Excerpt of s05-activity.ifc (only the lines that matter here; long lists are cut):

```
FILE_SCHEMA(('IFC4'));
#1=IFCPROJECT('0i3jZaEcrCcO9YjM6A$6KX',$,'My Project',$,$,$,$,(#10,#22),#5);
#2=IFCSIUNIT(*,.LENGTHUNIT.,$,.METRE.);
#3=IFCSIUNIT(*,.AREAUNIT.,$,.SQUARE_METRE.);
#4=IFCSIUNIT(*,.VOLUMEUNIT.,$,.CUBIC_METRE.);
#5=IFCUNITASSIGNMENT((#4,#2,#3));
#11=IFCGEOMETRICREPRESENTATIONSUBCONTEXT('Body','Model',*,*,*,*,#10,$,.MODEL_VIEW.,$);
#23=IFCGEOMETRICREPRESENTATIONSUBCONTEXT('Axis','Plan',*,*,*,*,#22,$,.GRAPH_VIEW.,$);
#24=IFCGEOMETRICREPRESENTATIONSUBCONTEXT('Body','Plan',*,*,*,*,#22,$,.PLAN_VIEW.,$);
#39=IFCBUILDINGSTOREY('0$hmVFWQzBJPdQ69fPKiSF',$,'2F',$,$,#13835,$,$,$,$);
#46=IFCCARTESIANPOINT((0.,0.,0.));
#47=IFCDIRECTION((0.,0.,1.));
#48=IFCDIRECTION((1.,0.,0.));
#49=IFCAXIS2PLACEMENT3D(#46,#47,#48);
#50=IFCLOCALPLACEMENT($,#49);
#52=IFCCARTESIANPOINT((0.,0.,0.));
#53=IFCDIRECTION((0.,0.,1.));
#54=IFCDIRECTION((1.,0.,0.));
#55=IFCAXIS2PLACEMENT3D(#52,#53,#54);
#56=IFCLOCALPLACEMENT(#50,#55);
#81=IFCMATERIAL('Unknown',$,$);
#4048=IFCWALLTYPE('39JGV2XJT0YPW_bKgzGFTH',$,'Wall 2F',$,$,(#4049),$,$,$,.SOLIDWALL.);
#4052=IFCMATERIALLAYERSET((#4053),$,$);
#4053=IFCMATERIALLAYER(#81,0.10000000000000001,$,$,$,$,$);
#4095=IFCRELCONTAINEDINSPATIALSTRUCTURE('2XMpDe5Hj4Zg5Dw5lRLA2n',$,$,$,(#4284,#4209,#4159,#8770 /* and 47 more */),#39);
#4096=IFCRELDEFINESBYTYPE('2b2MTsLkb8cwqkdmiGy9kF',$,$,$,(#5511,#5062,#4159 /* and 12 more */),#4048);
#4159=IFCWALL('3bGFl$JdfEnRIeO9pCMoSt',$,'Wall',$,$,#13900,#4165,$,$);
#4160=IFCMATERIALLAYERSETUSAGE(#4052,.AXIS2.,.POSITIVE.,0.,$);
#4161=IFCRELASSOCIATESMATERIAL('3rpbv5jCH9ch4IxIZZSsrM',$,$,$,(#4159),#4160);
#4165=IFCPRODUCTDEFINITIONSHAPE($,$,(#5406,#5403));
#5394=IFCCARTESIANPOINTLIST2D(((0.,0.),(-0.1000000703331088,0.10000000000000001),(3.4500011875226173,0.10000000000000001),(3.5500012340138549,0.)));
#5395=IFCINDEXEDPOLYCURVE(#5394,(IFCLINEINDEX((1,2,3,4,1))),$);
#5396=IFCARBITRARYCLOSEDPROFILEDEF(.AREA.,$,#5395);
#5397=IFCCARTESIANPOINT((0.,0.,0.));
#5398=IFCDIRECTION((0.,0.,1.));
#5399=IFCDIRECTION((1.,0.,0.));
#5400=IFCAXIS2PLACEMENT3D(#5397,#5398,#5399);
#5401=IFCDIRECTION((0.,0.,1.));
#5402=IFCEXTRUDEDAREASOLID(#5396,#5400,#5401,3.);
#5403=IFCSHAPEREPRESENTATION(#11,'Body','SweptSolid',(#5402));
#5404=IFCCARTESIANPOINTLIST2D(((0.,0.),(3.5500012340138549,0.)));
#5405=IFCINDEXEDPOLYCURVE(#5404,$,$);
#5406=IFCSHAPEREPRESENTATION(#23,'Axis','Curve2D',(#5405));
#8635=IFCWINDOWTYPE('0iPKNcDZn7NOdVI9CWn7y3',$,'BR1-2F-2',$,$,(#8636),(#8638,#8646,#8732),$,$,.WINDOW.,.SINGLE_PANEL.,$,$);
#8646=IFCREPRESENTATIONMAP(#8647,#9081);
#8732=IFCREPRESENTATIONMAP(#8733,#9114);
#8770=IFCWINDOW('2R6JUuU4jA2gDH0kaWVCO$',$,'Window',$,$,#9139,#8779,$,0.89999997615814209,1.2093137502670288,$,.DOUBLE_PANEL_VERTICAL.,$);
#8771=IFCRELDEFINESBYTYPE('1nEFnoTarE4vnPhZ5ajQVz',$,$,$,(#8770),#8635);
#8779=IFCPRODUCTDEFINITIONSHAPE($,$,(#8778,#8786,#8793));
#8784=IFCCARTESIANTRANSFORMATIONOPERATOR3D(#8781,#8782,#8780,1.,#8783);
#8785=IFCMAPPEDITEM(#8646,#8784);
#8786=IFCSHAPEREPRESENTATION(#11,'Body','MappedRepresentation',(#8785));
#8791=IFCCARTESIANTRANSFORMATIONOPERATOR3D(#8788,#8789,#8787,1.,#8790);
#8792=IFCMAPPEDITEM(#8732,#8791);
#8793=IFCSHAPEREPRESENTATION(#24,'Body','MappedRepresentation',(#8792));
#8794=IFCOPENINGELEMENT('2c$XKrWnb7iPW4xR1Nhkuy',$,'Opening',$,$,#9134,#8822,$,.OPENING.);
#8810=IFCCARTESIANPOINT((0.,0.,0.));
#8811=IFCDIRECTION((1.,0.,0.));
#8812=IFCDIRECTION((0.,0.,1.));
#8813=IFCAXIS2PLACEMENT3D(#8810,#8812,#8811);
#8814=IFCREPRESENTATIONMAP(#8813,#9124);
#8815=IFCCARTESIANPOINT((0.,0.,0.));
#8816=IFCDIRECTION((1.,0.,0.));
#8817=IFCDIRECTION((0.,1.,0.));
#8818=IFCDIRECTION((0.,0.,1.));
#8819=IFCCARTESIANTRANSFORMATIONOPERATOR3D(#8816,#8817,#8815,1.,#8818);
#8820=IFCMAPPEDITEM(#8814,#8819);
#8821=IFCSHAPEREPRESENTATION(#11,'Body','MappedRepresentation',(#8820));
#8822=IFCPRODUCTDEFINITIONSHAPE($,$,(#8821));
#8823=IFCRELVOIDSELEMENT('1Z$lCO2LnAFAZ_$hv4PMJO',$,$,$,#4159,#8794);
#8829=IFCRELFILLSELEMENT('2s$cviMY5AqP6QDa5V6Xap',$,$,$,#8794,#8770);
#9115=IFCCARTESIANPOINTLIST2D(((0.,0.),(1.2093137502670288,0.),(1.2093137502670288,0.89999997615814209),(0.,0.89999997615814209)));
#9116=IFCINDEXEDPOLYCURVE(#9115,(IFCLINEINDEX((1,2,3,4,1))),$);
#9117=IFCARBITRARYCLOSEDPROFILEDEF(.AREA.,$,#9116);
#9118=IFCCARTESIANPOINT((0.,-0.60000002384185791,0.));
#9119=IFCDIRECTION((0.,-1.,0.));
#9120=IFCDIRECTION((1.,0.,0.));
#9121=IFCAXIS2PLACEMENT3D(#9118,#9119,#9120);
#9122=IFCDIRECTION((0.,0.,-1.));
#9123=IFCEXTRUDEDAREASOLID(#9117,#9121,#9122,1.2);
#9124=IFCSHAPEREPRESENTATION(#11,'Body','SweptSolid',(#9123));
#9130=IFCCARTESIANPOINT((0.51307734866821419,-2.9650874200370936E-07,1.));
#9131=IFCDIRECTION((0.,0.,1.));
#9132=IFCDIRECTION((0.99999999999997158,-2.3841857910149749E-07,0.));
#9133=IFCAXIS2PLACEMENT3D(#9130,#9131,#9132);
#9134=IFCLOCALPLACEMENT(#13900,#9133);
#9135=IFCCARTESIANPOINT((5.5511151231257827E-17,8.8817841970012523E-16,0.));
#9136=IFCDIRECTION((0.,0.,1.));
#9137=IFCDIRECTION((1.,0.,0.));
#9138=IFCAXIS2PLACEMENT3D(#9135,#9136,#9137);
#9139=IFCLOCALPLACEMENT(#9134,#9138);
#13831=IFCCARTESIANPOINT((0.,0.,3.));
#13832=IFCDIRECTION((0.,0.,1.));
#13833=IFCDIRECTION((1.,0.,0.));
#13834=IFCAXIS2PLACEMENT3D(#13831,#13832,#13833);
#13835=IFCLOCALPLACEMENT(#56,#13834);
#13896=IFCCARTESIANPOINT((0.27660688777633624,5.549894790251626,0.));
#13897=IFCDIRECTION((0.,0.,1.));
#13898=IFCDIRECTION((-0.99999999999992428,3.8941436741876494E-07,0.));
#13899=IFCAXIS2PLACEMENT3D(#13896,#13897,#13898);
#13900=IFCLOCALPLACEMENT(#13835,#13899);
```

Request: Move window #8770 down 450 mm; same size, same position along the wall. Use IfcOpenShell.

```python
import numpy as np
import ifcopenshell
import ifcopenshell.api.geometry
import ifcopenshell.util.placement
import ifcopenshell.util.unit

model = ifcopenshell.open("s05-activity.ifc")
unit_scale = ifcopenshell.util.unit.calculate_unit_scale(model)

window = model.by_guid("2R6JUuU4jA2gDH0kaWVCO$")
opening = window.FillsVoids[0].RelatingOpeningElement
dz = -0.45

shift = np.array([0.0, 0.0, dz])
# The window is placed relative to its opening, so it follows when the opening moves.
matrix = ifcopenshell.util.placement.get_local_placement(opening.ObjectPlacement)
matrix[:3, 3] += shift
ifcopenshell.api.geometry.edit_object_placement(
    model, product=opening, matrix=matrix, is_si=False, should_transform_children=True
)

print(f"moved by {dz * unit_scale:+.3f} m")

model.write("s05-activity-out.ifc")
```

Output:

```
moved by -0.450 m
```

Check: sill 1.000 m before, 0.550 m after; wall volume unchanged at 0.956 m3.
